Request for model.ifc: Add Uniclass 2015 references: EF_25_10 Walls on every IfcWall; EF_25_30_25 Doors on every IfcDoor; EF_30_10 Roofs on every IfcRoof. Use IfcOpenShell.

First a look at what the model holds.

```python
import ifcopenshell

model = ifcopenshell.open("model.ifc")
print(model.schema)
print("classifications:", [c.Name for c in model.by_type("IfcClassification")])
for ifc_class in ("IfcDoor", "IfcRoof", "IfcStair", "IfcWall", "IfcWindow"):
    print(ifc_class, len(model.by_type(ifc_class)))
```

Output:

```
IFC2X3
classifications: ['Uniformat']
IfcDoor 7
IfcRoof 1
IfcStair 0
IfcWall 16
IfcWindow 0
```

```python
import ifcopenshell
import ifcopenshell.api.classification

model = ifcopenshell.open("model.ifc")

# IFC2X3 requires Source and Edition and has no link from the project to the system.
system = model.create_entity("IfcClassification", Source="NBS", Edition="2015", Name="Uniclass 2015")

codes = {
    "IfcWall": ("EF_25_10", "Walls"),
    "IfcDoor": ("EF_25_30_25", "Doors"),
    "IfcRoof": ("EF_30_10", "Roofs"),
}
for ifc_class, (code, name) in codes.items():
    products = model.by_type(ifc_class)
    ifcopenshell.api.classification.add_reference(
        model, products=products, classification=system, identification=code, name=name
    )
    print(code, len(products))

model.write("model-out.ifc")
```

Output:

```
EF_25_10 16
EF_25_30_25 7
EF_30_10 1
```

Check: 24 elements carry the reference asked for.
